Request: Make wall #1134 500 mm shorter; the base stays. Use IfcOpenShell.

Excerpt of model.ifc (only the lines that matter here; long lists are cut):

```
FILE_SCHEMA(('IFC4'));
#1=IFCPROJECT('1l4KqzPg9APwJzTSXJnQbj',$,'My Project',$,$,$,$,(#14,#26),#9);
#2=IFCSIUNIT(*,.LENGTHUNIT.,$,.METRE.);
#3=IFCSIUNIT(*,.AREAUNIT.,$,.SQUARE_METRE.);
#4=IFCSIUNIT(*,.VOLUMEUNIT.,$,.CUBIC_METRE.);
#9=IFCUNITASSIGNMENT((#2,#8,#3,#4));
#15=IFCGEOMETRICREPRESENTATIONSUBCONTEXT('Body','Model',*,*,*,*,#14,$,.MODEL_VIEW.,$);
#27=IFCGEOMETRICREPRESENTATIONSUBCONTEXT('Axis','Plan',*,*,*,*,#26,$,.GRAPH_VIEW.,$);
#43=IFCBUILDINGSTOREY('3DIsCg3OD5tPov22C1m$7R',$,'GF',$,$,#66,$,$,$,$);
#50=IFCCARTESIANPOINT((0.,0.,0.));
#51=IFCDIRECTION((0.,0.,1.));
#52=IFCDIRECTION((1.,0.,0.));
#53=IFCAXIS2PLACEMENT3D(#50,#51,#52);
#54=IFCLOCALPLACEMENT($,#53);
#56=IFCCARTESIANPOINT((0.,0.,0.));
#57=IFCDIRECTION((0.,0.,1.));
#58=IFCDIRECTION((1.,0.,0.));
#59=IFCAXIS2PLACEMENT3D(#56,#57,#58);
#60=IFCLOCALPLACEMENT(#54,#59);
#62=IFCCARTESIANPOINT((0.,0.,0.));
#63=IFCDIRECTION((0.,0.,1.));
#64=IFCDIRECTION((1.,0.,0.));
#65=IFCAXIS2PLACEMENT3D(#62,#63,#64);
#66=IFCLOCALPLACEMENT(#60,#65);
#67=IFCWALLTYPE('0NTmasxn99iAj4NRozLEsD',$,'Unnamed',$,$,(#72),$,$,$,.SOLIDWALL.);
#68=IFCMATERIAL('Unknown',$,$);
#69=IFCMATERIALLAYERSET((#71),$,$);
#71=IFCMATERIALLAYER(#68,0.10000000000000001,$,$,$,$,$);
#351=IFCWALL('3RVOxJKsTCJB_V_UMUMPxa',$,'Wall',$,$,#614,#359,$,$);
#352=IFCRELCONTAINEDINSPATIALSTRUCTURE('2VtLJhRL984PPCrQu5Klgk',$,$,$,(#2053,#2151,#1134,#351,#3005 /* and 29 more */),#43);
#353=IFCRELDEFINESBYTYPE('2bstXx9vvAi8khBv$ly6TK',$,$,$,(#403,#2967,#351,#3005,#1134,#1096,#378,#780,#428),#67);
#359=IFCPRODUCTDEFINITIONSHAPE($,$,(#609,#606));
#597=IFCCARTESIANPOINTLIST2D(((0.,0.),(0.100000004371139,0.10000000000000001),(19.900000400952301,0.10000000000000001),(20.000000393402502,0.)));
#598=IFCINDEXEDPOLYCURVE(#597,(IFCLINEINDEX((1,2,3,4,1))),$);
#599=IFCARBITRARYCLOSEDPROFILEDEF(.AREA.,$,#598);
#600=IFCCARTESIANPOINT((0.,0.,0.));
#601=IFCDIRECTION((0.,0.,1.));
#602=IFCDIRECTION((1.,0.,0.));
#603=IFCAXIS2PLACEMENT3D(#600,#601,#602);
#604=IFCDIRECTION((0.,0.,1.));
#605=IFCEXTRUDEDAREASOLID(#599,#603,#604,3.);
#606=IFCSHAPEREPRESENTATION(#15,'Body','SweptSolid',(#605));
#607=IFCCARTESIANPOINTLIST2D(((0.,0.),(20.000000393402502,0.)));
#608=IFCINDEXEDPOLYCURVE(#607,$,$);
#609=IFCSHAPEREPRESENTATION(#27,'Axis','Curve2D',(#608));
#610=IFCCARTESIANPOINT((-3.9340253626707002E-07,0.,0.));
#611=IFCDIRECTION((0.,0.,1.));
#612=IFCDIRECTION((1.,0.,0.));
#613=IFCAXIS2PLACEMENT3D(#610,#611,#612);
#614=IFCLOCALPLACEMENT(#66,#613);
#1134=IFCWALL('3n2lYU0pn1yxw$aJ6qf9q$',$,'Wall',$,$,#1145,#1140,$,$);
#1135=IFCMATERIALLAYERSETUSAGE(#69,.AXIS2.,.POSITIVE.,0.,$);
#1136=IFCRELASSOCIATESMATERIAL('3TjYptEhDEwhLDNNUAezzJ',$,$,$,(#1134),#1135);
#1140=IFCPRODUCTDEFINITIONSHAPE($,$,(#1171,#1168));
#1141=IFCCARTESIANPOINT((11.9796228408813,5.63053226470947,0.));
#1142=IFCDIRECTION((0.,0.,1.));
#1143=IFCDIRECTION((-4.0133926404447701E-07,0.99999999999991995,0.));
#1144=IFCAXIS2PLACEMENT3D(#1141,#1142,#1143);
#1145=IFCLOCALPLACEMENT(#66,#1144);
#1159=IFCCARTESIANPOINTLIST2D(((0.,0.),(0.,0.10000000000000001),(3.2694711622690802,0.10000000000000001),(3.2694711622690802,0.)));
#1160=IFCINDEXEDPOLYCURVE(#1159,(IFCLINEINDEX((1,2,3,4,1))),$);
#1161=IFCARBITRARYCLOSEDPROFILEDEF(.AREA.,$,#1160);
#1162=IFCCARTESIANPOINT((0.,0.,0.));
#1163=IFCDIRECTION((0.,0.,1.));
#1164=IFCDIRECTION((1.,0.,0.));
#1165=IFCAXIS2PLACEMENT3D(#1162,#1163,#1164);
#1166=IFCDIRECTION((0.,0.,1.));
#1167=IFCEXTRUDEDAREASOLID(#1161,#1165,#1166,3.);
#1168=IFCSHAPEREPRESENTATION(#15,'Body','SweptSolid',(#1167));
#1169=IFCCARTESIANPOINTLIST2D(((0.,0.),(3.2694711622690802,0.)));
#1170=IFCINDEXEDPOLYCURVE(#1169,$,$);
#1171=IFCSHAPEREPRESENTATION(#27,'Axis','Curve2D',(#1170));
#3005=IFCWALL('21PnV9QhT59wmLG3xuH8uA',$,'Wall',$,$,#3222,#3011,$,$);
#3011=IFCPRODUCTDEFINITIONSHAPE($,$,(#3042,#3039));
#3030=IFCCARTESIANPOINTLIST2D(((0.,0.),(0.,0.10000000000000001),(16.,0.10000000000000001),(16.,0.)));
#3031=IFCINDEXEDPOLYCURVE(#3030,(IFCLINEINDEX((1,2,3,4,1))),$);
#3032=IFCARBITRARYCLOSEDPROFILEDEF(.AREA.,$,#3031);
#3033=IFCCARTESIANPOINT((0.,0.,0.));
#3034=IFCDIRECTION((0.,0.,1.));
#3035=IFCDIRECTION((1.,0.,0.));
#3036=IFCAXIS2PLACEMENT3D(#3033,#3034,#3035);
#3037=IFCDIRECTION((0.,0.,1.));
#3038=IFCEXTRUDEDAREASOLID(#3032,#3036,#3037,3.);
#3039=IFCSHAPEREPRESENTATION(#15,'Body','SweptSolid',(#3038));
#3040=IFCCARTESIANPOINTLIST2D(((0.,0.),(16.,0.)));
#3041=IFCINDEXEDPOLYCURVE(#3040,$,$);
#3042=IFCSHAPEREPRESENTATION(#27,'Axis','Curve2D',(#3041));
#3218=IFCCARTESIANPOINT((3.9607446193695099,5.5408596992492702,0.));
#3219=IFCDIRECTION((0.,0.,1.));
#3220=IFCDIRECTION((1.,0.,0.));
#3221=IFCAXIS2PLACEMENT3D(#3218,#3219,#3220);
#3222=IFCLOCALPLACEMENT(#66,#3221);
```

```python
import ifcopenshell
import ifcopenshell.geom
import ifcopenshell.util.representation
import ifcopenshell.util.shape

model = ifcopenshell.open("model.ifc")
settings = ifcopenshell.geom.settings()


def volume(element):
    """Net volume in cubic metres, openings subtracted."""
    shape = ifcopenshell.geom.create_shape(settings, element)
    return ifcopenshell.util.shape.get_volume(shape.geometry)


wall = model.by_guid("3n2lYU0pn1yxw$aJ6qf9q$")
before = volume(wall)

body = ifcopenshell.util.representation.get_representation(wall, "Model", "Body")
solid = body.Items[0]
old_height = solid.Depth
solid.Depth -= 0.5
after = volume(wall)

print(f"height {old_height:g} -> {solid.Depth:g}, volume {before:.3f} -> {after:.3f} m3")

model.write("model_edited.ifc")
```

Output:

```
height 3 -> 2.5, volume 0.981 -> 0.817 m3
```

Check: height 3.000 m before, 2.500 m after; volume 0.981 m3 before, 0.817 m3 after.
